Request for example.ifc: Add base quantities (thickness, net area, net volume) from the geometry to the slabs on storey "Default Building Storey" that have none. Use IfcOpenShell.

First a look at what the model holds.

```python
import ifcopenshell
import ifcopenshell.util.element
import ifcopenshell.util.unit

model = ifcopenshell.open("example.ifc")
print(model.schema)
for unit_type in ("LENGTHUNIT", "AREAUNIT", "VOLUMEUNIT"):
    print(unit_type, ifcopenshell.util.unit.calculate_unit_scale(model, unit_type))
storey = next(s for s in model.by_type("IfcBuildingStorey") if s.Name == "Default Building Storey")
slabs = [e for e in ifcopenshell.util.element.get_decomposition(storey) if e.is_a("IfcSlab")]
for e in sorted(slabs, key=lambda e: e.id()):
    print(e.id(), e.is_a(), e.Name, list(ifcopenshell.util.element.get_psets(e, qtos_only=True)), sep=" | ")
```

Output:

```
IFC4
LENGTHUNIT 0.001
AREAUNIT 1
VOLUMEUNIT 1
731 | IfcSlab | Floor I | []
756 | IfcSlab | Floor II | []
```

```python
import ifcopenshell
import ifcopenshell.api.pset
import ifcopenshell.geom
import ifcopenshell.util.element
import ifcopenshell.util.shape
import ifcopenshell.util.unit

model = ifcopenshell.open("example.ifc")
unit_scale = ifcopenshell.util.unit.calculate_unit_scale(model)
area_scale = ifcopenshell.util.unit.calculate_unit_scale(model, "AREAUNIT")
volume_scale = ifcopenshell.util.unit.calculate_unit_scale(model, "VOLUMEUNIT")
settings = ifcopenshell.geom.settings()

storey = next(s for s in model.by_type("IfcBuildingStorey") if s.Name == "Default Building Storey")
slabs = [e for e in ifcopenshell.util.element.get_decomposition(storey) if e.is_a("IfcSlab")]

for e in sorted(slabs, key=lambda e: e.id()):
    if ifcopenshell.util.element.get_psets(e, qtos_only=True, should_inherit=False):
        continue
    # Geometry comes back in metres, in the element's own axes.
    shape = ifcopenshell.geom.create_shape(settings, e)
    values = {
        "Width": ifcopenshell.util.shape.get_z(shape.geometry) / unit_scale,
        "NetArea": ifcopenshell.util.shape.get_footprint_area(shape.geometry) / area_scale,
        "NetVolume": ifcopenshell.util.shape.get_volume(shape.geometry) / volume_scale,
    }
    qto = ifcopenshell.api.pset.add_qto(model, product=e, name="Qto_SlabBaseQuantities")
    ifcopenshell.api.pset.edit_qto(model, qto=qto, properties=values)
    print(e.id(), {k: round(v, 3) for k, v in values.items()})

model.write("example-out.ifc")
```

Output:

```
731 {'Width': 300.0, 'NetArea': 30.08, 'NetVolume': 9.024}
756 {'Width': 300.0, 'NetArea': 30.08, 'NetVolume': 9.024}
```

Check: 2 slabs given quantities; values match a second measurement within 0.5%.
